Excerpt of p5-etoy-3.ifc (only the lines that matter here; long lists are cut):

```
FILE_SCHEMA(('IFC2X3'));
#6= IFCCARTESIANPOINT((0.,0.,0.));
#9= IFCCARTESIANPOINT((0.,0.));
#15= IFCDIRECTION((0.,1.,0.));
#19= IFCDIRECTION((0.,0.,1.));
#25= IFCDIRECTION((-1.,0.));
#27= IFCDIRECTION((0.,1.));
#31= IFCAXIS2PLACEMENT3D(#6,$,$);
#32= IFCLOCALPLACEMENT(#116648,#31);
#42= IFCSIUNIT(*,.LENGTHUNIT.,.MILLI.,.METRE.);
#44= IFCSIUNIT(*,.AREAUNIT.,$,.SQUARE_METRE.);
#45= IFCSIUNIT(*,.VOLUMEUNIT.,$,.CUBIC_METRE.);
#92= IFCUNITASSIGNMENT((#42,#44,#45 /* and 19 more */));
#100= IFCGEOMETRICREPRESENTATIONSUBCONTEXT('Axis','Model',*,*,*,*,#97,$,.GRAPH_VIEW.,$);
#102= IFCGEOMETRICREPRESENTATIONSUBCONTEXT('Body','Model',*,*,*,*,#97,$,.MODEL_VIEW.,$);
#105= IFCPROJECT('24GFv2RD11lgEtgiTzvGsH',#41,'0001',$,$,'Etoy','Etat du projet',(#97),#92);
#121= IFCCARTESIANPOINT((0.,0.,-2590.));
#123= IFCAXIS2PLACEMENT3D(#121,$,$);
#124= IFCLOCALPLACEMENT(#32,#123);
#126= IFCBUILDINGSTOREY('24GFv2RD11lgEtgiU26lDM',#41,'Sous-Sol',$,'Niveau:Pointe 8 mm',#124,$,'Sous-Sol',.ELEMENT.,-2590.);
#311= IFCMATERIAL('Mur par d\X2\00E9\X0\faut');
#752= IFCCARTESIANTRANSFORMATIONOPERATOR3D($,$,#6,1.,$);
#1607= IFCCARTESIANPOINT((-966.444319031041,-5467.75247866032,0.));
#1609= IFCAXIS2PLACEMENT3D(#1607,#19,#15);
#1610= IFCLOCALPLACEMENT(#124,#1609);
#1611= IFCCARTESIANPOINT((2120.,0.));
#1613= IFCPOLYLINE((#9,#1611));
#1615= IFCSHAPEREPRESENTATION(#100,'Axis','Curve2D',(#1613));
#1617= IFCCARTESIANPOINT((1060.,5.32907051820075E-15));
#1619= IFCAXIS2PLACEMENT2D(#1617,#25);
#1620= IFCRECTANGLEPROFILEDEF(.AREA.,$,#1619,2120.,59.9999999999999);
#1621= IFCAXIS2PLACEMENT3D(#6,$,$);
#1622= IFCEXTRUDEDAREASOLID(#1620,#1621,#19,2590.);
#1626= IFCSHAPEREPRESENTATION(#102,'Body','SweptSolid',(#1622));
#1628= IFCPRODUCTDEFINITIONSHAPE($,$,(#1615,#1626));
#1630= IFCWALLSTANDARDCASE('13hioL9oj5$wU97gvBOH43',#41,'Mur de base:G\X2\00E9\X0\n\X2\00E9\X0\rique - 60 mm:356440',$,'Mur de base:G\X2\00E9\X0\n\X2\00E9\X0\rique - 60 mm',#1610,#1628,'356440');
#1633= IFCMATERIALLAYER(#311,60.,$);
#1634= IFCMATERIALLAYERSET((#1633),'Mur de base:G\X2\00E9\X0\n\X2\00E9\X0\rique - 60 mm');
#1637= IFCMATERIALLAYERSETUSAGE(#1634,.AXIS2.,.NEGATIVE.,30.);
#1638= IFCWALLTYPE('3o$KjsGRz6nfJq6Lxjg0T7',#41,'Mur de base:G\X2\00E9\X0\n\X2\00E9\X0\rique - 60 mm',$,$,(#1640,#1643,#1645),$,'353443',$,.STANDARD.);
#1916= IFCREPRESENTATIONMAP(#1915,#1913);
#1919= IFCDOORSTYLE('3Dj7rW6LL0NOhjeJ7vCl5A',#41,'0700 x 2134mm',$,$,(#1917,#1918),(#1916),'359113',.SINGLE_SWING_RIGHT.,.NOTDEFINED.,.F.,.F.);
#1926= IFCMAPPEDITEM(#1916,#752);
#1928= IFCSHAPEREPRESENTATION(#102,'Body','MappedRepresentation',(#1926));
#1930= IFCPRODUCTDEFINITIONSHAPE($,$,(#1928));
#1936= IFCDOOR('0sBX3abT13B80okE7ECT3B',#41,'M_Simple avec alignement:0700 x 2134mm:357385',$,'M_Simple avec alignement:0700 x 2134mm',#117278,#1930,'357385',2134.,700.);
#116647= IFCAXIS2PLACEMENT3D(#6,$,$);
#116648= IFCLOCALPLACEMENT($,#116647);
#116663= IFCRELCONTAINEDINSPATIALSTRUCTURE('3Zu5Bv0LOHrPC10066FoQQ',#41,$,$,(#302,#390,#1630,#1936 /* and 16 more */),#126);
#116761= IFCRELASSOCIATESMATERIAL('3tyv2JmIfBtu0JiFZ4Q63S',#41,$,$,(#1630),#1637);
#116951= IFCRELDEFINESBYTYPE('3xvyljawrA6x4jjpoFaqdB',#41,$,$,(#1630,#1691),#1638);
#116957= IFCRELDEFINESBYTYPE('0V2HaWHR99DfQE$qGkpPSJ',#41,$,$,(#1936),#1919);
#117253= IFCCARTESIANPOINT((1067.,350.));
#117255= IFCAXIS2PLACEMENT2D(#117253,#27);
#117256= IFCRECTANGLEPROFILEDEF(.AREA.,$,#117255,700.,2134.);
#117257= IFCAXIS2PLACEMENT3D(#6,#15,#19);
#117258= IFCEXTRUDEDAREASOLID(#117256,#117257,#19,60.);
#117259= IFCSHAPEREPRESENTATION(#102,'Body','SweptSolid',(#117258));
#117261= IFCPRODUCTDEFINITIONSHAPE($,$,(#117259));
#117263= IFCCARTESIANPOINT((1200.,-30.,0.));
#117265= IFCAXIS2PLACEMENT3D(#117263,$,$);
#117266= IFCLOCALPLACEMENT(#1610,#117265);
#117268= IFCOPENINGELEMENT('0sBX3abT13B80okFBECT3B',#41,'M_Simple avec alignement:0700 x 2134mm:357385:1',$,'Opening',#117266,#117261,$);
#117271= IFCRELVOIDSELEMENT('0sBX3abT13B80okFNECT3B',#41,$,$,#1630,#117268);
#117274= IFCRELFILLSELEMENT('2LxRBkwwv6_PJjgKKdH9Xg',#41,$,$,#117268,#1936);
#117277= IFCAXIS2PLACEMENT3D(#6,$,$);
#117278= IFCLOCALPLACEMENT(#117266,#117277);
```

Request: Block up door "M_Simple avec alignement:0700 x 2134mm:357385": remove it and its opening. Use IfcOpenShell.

```python
import ifcopenshell
import ifcopenshell.api.feature
import ifcopenshell.api.root
import ifcopenshell.geom
import ifcopenshell.util.shape

model = ifcopenshell.open("p5-etoy-3.ifc")
settings = ifcopenshell.geom.settings()


def volume(element):
    """Net volume in cubic metres, openings subtracted."""
    shape = ifcopenshell.geom.create_shape(settings, element)
    return ifcopenshell.util.shape.get_volume(shape.geometry)


door = model.by_id(1936)
opening = door.FillsVoids[0].RelatingOpeningElement
wall = opening.VoidsElements[0].RelatingBuildingElement
before = volume(wall)

ifcopenshell.api.root.remove_product(model, product=door)
ifcopenshell.api.feature.remove_feature(model, feature=opening)

after = volume(wall)

print(f"wall volume {before:.3f} -> {after:.3f} m3")

model.write("p5-etoy-3_edited.ifc")
```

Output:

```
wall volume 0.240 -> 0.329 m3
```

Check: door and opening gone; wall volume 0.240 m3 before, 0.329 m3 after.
